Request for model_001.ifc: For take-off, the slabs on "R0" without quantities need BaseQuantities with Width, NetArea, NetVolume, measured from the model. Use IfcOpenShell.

First a look at what the model holds.

```python
import ifcopenshell
import ifcopenshell.util.element
import ifcopenshell.util.unit

model = ifcopenshell.open("model_001.ifc")
print(model.schema)
for unit_type in ("LENGTHUNIT", "AREAUNIT", "VOLUMEUNIT"):
    print(unit_type, ifcopenshell.util.unit.calculate_unit_scale(model, unit_type))
storey = next(s for s in model.by_type("IfcBuildingStorey") if s.Name == "R0")
slabs = [e for e in ifcopenshell.util.element.get_decomposition(storey) if e.is_a("IfcSlab")]
for e in sorted(slabs, key=lambda e: e.id()):
    print(e.id(), e.is_a(), e.Name, list(ifcopenshell.util.element.get_psets(e, qtos_only=True)), sep=" | ")
```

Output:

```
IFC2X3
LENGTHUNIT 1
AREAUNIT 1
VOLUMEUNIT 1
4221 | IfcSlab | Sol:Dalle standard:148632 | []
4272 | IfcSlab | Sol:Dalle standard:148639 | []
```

```python
import ifcopenshell
import ifcopenshell.api.pset
import ifcopenshell.geom
import ifcopenshell.util.element
import ifcopenshell.util.shape
import ifcopenshell.util.unit

model = ifcopenshell.open("model_001.ifc")
unit_scale = ifcopenshell.util.unit.calculate_unit_scale(model)
area_scale = ifcopenshell.util.unit.calculate_unit_scale(model, "AREAUNIT")
volume_scale = ifcopenshell.util.unit.calculate_unit_scale(model, "VOLUMEUNIT")
settings = ifcopenshell.geom.settings()

storey = next(s for s in model.by_type("IfcBuildingStorey") if s.Name == "R0")
slabs = [e for e in ifcopenshell.util.element.get_decomposition(storey) if e.is_a("IfcSlab")]

for e in sorted(slabs, key=lambda e: e.id()):
    if ifcopenshell.util.element.get_psets(e, qtos_only=True, should_inherit=False):
        continue
    # Geometry comes back in metres, in the element's own axes.
    shape = ifcopenshell.geom.create_shape(settings, e)
    values = {
        "Width": ifcopenshell.util.shape.get_z(shape.geometry) / unit_scale,
        "NetArea": ifcopenshell.util.shape.get_footprint_area(shape.geometry) / area_scale,
        "NetVolume": ifcopenshell.util.shape.get_volume(shape.geometry) / volume_scale,
    }
    qto = ifcopenshell.api.pset.add_qto(model, product=e, name="BaseQuantities")
    ifcopenshell.api.pset.edit_qto(model, qto=qto, properties=values)
    print(e.id(), {k: round(v, 3) for k, v in values.items()})

model.write("model_001-out.ifc")
```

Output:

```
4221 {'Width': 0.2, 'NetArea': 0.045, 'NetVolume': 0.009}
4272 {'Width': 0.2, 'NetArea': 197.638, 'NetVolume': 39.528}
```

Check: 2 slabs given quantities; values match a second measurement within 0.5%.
